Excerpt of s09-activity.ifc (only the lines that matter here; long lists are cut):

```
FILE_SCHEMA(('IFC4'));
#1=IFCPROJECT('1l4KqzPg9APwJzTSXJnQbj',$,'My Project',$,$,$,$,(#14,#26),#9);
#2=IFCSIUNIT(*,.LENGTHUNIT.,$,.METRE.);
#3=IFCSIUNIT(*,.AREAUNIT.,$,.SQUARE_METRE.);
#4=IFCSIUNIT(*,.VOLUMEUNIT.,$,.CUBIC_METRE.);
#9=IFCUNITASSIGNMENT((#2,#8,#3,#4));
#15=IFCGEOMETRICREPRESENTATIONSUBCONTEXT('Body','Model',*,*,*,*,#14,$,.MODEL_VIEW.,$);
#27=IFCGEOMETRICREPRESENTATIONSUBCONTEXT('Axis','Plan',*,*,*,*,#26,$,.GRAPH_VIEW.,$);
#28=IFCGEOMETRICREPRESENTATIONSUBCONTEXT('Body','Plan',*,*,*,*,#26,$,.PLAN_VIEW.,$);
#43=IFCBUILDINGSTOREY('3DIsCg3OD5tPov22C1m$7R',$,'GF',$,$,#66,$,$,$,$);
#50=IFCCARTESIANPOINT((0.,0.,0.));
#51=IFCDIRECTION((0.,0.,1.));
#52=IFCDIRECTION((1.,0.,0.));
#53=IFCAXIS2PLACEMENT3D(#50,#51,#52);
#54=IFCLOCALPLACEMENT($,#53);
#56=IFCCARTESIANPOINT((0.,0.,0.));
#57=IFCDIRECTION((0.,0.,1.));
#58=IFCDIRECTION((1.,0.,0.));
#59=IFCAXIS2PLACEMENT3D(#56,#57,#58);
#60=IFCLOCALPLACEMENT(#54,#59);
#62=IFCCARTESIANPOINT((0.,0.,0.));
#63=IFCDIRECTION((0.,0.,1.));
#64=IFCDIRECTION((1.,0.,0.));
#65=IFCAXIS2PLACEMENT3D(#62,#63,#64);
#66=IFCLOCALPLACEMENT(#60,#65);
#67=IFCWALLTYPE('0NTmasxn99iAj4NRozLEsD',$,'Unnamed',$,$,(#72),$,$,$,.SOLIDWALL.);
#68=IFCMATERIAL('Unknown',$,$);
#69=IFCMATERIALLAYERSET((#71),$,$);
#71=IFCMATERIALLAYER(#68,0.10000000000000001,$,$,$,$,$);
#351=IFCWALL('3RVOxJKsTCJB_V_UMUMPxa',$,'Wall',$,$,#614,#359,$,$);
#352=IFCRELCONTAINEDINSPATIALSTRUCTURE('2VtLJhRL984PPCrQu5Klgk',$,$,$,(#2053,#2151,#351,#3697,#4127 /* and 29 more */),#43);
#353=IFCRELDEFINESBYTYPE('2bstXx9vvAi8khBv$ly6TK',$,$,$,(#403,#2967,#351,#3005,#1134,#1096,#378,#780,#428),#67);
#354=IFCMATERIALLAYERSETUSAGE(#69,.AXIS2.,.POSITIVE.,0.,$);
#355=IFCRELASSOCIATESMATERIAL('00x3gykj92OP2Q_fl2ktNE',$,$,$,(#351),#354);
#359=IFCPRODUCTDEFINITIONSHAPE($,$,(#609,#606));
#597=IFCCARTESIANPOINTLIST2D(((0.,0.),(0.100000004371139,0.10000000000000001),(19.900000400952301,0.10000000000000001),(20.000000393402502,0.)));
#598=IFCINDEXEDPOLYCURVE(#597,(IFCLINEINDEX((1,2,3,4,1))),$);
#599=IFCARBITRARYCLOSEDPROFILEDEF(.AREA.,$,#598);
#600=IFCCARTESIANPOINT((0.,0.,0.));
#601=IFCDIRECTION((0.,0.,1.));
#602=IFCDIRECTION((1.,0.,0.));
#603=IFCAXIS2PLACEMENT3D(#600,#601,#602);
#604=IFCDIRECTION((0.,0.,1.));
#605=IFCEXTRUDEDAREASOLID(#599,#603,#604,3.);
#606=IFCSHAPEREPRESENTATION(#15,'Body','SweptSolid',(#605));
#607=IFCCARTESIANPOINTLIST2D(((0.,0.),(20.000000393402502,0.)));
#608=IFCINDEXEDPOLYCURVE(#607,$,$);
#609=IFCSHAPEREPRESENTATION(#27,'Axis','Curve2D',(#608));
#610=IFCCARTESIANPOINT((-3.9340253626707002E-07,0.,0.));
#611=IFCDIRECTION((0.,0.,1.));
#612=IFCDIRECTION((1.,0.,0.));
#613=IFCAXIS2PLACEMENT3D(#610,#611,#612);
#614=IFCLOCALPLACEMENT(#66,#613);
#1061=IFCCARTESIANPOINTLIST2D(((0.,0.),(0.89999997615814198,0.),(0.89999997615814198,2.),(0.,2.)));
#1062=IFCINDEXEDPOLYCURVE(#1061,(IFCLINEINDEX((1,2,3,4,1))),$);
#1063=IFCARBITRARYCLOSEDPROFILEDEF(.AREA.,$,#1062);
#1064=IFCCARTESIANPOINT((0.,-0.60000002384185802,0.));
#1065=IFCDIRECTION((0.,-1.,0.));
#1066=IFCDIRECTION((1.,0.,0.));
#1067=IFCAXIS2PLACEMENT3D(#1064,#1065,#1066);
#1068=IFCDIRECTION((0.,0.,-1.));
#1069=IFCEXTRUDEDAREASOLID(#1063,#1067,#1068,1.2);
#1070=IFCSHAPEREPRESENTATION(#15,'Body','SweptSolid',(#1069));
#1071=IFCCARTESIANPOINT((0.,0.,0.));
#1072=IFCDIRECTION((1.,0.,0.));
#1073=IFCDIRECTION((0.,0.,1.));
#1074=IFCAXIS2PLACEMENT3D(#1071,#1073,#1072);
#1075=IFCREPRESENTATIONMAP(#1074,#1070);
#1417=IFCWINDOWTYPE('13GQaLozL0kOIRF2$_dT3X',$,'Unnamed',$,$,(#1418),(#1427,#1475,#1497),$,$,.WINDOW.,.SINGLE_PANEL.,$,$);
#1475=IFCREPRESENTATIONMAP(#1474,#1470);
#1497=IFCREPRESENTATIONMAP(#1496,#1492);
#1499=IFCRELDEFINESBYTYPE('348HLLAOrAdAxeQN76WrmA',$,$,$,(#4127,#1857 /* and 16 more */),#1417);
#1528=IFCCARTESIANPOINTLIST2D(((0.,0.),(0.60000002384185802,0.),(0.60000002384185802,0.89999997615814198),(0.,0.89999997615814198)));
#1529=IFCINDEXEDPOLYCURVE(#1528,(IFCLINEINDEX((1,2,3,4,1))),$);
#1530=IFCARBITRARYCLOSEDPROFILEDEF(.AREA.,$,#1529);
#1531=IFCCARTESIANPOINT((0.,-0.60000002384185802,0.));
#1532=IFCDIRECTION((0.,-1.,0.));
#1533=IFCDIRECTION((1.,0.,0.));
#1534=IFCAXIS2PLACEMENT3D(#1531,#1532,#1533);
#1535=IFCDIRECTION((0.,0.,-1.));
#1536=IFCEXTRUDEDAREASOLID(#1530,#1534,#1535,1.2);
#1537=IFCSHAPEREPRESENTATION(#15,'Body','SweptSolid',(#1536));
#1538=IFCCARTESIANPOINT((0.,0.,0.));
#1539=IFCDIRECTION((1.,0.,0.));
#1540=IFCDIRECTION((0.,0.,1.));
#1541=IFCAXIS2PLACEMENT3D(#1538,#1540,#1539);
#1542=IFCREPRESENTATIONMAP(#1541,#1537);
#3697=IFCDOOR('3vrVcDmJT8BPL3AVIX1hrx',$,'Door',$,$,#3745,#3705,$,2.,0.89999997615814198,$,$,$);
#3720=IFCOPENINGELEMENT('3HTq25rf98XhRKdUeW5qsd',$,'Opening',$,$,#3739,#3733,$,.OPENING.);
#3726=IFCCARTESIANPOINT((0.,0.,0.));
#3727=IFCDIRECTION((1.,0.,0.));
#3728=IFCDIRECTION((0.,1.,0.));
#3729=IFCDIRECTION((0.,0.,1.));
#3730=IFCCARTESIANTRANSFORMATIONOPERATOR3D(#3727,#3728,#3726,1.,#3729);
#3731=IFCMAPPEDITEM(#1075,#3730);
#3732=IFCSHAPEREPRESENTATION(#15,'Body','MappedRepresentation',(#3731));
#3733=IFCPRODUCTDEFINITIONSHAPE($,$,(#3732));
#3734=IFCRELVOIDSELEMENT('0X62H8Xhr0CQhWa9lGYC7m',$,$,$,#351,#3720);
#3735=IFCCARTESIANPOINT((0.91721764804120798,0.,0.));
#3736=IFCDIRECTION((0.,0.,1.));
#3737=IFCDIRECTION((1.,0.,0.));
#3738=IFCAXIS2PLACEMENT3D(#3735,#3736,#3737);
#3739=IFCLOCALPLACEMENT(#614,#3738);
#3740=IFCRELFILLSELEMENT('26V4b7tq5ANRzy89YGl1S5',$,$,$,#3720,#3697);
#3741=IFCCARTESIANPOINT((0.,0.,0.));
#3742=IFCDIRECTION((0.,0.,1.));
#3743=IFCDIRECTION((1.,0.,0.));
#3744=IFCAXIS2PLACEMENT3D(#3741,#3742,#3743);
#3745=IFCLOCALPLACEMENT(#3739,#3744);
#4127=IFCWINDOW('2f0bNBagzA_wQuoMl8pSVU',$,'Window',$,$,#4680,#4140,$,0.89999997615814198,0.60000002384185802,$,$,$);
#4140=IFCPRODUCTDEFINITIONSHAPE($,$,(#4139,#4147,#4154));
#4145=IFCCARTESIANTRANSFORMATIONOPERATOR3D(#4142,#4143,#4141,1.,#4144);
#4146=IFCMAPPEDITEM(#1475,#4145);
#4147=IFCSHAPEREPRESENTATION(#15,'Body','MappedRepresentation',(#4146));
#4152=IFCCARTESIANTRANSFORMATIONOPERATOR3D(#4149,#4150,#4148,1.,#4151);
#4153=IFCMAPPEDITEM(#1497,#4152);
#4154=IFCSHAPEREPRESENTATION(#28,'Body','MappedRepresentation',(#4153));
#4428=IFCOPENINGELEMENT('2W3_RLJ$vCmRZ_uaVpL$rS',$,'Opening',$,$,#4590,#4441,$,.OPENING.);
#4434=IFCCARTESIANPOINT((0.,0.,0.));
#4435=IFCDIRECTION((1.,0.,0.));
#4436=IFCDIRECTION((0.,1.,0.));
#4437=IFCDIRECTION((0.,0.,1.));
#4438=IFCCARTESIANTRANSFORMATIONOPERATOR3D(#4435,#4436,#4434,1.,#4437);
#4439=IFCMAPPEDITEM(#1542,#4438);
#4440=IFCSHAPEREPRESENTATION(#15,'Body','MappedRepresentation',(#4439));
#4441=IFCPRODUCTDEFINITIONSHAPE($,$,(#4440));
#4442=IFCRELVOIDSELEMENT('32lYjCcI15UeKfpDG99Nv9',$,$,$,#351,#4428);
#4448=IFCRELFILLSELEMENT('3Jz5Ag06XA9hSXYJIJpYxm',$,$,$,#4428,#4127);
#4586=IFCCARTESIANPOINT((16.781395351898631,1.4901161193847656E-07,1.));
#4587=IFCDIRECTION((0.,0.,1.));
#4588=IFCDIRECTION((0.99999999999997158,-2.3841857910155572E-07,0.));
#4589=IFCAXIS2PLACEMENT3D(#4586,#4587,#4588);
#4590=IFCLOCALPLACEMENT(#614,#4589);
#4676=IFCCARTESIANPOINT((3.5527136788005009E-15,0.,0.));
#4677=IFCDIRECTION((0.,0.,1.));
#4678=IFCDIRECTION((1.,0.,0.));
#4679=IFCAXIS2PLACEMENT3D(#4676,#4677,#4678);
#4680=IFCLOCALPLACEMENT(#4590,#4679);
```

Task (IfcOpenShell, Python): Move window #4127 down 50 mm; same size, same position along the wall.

```python
import numpy as np
import ifcopenshell
import ifcopenshell.api.geometry
import ifcopenshell.util.placement
import ifcopenshell.util.unit

model = ifcopenshell.open("s09-activity.ifc")
unit_scale = ifcopenshell.util.unit.calculate_unit_scale(model)

window = model.by_guid("2f0bNBagzA_wQuoMl8pSVU")
opening = window.FillsVoids[0].RelatingOpeningElement
dz = -0.05 / unit_scale

shift = np.array([0.0, 0.0, dz])
# The window is placed relative to its opening, so it follows when the opening moves.
matrix = ifcopenshell.util.placement.get_local_placement(opening.ObjectPlacement)
matrix[:3, 3] += shift
ifcopenshell.api.geometry.edit_object_placement(
    model, product=opening, matrix=matrix, is_si=False, should_transform_children=True
)

print(f"moved by {dz * unit_scale:+.3f} m")

model.write("s09-activity_v2.ifc")
```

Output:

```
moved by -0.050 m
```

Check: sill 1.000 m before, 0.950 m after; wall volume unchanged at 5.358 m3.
